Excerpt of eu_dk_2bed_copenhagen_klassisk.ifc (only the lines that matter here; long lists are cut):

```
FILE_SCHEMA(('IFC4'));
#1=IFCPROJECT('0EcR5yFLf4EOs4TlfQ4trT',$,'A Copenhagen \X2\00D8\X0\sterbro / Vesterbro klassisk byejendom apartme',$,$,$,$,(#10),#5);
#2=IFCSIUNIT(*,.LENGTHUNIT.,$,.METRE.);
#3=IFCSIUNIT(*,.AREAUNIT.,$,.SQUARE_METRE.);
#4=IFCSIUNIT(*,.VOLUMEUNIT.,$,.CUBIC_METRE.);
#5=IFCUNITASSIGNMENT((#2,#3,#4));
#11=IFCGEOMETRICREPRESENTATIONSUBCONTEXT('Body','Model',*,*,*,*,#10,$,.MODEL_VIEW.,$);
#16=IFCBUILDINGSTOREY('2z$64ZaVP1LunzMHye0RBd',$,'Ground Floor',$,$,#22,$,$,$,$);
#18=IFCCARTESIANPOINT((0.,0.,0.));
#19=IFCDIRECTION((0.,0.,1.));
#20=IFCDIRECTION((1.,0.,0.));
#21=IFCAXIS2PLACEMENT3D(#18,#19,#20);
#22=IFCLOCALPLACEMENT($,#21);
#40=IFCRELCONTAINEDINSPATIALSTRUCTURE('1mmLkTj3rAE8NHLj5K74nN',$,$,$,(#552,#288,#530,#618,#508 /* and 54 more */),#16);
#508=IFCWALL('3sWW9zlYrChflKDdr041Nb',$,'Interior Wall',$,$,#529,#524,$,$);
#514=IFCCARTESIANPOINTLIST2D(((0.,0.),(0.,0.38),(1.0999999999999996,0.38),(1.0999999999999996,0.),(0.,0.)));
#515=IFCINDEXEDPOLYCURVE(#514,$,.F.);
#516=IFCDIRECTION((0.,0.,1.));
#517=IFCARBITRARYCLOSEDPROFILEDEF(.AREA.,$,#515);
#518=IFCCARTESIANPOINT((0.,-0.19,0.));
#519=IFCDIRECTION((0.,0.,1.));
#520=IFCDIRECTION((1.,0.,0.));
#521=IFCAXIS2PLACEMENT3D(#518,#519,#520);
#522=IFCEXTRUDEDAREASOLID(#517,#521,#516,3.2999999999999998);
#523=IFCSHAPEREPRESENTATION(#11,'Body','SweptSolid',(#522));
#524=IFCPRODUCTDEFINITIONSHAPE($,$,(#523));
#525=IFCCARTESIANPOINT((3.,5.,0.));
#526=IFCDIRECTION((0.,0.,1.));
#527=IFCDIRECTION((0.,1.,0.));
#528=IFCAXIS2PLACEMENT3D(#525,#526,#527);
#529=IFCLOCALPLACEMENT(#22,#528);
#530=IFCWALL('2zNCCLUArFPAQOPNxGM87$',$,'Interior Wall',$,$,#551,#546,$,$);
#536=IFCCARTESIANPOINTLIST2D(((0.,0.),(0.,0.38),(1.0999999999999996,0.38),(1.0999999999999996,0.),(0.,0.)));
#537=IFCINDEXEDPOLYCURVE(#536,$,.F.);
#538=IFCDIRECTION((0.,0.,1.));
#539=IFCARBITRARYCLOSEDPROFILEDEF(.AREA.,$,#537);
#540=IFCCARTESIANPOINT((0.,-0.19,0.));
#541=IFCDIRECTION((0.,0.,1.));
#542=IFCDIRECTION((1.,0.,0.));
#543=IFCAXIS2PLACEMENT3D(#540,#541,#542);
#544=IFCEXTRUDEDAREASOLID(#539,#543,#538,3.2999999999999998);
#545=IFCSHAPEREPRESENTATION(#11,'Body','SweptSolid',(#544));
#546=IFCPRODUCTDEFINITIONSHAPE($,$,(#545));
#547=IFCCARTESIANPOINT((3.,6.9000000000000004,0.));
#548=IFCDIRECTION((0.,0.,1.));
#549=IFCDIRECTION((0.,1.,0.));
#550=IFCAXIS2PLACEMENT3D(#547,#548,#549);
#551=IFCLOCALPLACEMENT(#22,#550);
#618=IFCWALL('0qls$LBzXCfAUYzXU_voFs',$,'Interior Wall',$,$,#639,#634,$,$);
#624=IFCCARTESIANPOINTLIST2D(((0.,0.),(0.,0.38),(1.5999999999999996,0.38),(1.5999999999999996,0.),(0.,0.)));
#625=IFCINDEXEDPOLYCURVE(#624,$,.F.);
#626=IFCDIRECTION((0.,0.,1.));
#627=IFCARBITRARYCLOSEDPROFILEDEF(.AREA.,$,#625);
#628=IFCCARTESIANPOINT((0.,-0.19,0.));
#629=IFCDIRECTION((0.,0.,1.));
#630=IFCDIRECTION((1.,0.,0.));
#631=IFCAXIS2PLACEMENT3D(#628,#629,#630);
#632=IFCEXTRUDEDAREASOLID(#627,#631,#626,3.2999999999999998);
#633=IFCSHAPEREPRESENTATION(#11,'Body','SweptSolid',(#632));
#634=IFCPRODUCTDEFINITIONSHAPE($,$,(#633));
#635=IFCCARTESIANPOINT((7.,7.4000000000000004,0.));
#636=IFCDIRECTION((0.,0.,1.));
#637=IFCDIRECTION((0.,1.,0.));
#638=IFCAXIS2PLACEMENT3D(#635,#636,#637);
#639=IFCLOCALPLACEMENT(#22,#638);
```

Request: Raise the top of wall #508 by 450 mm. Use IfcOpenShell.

```python
import ifcopenshell
import ifcopenshell.geom
import ifcopenshell.util.representation
import ifcopenshell.util.shape
import ifcopenshell.util.unit

model = ifcopenshell.open("eu_dk_2bed_copenhagen_klassisk.ifc")
unit_scale = ifcopenshell.util.unit.calculate_unit_scale(model)
settings = ifcopenshell.geom.settings()


def volume(element):
    """Net volume in cubic metres, openings subtracted."""
    shape = ifcopenshell.geom.create_shape(settings, element)
    return ifcopenshell.util.shape.get_volume(shape.geometry)


wall = model.by_id(508)
before = volume(wall)

body = ifcopenshell.util.representation.get_representation(wall, "Model", "Body")
solid = body.Items[0]
old_height = solid.Depth
solid.Depth += 0.45 / unit_scale
after = volume(wall)

print(f"height {old_height:g} -> {solid.Depth:g}, volume {before:.3f} -> {after:.3f} m3")

model.write("eu_dk_2bed_copenhagen_klassisk-out.ifc")
```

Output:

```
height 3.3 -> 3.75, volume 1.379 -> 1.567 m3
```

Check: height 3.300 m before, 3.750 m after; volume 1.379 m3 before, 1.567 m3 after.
